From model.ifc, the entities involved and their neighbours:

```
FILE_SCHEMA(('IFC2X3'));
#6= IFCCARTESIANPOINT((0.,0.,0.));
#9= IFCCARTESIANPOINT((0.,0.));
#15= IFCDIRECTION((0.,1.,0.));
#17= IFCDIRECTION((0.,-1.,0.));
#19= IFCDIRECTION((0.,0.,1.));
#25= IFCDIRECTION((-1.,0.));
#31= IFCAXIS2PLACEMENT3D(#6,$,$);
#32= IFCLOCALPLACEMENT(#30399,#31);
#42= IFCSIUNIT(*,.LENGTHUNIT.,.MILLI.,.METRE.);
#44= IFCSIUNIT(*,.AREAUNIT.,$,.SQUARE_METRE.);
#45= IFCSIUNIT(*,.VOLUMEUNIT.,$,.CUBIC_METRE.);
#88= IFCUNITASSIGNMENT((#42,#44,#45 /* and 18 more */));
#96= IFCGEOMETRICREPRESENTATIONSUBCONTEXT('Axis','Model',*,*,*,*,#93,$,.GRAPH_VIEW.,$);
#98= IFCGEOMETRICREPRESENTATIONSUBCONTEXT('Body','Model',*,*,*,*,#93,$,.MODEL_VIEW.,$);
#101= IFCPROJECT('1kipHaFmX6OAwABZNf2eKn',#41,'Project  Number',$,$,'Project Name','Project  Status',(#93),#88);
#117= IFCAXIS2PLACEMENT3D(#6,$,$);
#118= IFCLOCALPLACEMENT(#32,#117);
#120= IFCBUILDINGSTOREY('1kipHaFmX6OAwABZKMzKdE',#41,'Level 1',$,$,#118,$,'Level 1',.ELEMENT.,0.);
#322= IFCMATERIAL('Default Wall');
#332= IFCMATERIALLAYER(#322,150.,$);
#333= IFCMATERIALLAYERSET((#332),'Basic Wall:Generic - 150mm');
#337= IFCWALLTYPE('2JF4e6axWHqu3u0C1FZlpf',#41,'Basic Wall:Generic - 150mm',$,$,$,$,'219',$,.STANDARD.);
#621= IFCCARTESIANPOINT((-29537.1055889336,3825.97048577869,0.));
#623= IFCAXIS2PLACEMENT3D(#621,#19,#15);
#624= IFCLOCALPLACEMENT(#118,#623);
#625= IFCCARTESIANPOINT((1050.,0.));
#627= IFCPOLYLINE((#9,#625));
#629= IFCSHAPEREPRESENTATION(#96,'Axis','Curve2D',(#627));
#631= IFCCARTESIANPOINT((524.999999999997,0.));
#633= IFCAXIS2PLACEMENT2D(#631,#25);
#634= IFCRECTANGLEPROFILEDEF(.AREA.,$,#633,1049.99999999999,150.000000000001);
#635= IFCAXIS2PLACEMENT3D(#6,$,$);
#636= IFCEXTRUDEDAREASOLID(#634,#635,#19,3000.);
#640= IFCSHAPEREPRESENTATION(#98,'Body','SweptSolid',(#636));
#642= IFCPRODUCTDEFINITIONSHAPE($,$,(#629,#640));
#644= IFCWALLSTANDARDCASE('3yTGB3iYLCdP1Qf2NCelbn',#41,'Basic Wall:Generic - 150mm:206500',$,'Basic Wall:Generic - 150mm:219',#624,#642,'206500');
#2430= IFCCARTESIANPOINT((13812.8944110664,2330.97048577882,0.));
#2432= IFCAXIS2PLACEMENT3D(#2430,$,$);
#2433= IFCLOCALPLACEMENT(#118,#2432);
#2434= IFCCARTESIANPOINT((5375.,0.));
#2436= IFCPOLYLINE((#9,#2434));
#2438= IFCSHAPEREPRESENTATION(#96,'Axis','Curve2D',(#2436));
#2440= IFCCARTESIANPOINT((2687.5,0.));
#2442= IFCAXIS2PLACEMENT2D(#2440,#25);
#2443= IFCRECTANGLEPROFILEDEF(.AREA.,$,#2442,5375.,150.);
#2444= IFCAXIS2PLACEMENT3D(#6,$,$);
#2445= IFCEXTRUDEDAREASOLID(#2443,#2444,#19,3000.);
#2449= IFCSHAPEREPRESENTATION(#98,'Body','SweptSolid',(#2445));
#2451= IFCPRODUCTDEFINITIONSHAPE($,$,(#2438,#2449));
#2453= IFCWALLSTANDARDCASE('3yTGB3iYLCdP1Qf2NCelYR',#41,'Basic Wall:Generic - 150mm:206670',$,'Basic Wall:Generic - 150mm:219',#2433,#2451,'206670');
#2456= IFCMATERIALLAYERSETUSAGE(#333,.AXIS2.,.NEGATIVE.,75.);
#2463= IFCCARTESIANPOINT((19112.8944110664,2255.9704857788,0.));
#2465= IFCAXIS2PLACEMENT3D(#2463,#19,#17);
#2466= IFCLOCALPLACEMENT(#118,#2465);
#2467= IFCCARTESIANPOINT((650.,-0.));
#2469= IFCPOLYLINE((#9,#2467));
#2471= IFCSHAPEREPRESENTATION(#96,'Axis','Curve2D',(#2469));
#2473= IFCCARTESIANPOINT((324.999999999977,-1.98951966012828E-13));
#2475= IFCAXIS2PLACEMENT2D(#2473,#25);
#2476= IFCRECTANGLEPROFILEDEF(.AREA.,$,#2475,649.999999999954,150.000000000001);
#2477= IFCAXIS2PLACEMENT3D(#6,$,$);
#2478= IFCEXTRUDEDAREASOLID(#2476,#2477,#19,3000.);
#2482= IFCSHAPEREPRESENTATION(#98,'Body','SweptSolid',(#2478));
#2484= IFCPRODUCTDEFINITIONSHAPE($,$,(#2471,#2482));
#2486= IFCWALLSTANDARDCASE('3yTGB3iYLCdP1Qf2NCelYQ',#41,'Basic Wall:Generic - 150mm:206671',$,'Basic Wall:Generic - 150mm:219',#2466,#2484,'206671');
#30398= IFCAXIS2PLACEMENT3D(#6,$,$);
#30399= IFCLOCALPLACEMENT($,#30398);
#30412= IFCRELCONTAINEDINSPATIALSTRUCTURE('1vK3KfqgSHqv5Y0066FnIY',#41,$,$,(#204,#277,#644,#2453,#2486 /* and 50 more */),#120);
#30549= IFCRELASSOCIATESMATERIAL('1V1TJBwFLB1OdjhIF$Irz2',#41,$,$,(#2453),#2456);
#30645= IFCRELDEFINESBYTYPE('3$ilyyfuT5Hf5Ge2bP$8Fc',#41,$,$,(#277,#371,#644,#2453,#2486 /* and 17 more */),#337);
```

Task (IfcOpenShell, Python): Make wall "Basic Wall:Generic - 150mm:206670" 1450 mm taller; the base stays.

```python
import ifcopenshell
import ifcopenshell.geom
import ifcopenshell.util.representation
import ifcopenshell.util.shape

model = ifcopenshell.open("model.ifc")
settings = ifcopenshell.geom.settings()


def volume(element):
    """Net volume in cubic metres, openings subtracted."""
    shape = ifcopenshell.geom.create_shape(settings, element)
    return ifcopenshell.util.shape.get_volume(shape.geometry)


wall = model.by_guid("3yTGB3iYLCdP1Qf2NCelYR")
before = volume(wall)

body = ifcopenshell.util.representation.get_representation(wall, "Model", "Body")
solid = body.Items[0]
old_height = solid.Depth
solid.Depth += 1450.0
after = volume(wall)

print(f"height {old_height:g} -> {solid.Depth:g}, volume {before:.3f} -> {after:.3f} m3")

model.write("model_v2.ifc")
```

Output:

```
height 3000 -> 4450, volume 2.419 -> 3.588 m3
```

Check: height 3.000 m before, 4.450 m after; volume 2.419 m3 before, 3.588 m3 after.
